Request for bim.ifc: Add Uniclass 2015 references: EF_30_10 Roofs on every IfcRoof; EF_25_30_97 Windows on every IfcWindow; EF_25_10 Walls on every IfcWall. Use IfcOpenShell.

First a look at what the model holds.

```python
import ifcopenshell

model = ifcopenshell.open("bim.ifc")
print(model.schema)
print("classifications:", [c.Name for c in model.by_type("IfcClassification")])
for ifc_class in ("IfcDoor", "IfcRoof", "IfcStair", "IfcWall", "IfcWindow"):
    print(ifc_class, len(model.by_type(ifc_class)))
```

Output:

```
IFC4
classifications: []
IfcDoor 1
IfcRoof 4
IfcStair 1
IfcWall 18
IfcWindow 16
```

```python
import ifcopenshell
import ifcopenshell.api.classification

model = ifcopenshell.open("bim.ifc")

system = ifcopenshell.api.classification.add_classification(model, classification="Uniclass 2015")

codes = {
    "IfcRoof": ("EF_30_10", "Roofs"),
    "IfcWindow": ("EF_25_30_97", "Windows"),
    "IfcWall": ("EF_25_10", "Walls"),
}
for ifc_class, (code, name) in codes.items():
    products = model.by_type(ifc_class)
    ifcopenshell.api.classification.add_reference(
        model, products=products, classification=system, identification=code, name=name
    )
    print(code, len(products))

model.write("bim_edited.ifc")
```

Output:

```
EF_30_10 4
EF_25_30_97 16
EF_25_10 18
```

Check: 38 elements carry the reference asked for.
